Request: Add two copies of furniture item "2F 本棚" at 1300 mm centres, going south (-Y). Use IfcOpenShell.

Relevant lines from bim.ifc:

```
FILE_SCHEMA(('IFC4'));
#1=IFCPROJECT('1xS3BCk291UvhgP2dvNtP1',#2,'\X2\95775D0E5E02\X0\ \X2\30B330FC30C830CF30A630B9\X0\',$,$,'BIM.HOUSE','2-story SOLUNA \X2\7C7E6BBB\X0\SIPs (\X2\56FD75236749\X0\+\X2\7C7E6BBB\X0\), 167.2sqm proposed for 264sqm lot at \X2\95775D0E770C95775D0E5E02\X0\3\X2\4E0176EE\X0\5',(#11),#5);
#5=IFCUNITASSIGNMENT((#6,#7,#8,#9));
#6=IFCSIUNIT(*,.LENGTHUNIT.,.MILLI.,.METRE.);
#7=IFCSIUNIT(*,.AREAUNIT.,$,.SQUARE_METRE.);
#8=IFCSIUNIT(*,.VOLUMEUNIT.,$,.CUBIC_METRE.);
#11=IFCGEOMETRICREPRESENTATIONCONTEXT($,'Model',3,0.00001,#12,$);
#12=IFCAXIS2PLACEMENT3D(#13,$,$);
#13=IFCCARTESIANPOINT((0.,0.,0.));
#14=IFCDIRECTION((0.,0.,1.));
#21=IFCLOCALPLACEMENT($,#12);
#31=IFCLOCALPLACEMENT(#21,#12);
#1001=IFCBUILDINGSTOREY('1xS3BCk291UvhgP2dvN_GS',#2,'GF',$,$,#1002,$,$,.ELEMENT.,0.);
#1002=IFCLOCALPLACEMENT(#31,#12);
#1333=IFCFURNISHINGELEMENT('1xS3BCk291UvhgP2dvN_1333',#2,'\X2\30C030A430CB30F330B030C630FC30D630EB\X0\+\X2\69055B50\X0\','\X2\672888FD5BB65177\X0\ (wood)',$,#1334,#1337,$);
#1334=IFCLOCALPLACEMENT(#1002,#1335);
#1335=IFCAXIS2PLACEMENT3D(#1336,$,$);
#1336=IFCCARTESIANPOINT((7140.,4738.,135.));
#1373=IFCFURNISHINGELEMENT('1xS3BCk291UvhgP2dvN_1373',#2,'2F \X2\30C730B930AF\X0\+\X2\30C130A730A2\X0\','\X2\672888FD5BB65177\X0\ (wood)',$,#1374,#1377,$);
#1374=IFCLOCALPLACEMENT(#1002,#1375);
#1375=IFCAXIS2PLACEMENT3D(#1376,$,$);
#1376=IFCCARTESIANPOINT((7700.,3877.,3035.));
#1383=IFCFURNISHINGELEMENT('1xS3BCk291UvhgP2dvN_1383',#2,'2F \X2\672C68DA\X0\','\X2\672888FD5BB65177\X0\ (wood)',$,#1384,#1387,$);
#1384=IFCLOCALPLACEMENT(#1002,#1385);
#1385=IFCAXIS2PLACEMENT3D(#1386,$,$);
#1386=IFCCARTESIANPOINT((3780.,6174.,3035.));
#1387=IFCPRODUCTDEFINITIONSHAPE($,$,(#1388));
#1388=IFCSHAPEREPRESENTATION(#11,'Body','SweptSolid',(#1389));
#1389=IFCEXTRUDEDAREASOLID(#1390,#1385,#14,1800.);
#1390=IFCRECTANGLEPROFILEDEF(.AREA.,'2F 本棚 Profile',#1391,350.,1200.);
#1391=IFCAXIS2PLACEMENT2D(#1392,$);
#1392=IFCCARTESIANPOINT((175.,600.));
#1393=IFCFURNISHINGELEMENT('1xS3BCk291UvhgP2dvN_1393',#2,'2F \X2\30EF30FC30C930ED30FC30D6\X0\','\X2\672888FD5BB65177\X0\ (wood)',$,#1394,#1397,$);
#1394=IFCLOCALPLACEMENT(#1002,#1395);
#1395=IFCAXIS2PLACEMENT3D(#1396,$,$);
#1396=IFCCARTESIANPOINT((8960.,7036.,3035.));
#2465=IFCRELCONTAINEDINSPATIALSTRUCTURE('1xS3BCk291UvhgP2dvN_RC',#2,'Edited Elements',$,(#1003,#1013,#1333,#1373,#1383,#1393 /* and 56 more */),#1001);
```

```python
import numpy as np
import ifcopenshell
import ifcopenshell.api.geometry
import ifcopenshell.api.root
import ifcopenshell.util.element
import ifcopenshell.util.placement
import ifcopenshell.util.unit

model = ifcopenshell.open("bim.ifc")
unit_scale = ifcopenshell.util.unit.calculate_unit_scale(model)


def reuse_history(source, copy):
    """copy_class also copies each property set's owner history, people and application; keep the originals."""
    for rel in copy.IsDefinedBy:
        if rel.is_a("IfcRelDefinesByProperties") and (history := rel.RelatingPropertyDefinition.OwnerHistory):
            rel.RelatingPropertyDefinition.OwnerHistory = source.OwnerHistory
            ifcopenshell.util.element.remove_deep2(model, history)


source = model.by_guid("1xS3BCk291UvhgP2dvN_1383")
base = ifcopenshell.util.placement.get_local_placement(source.ObjectPlacement)
step = np.array([0.0, -1.0, 0.0]) * 1.3 / unit_scale

for i in range(1, 3):
    copy = ifcopenshell.api.root.copy_class(model, product=source)
    copy.Representation = ifcopenshell.util.element.copy_deep(
        model, source.Representation, exclude=["IfcGeometricRepresentationContext", "IfcRepresentationMap"]
    )
    reuse_history(source, copy)
    matrix = base.copy()
    matrix[:3, 3] += i * step
    print("added at", matrix[:3, 3].round(3) + 0.0)
    ifcopenshell.api.geometry.edit_object_placement(model, product=copy, matrix=matrix, is_si=False)

model.write("bim_rev.ifc")
```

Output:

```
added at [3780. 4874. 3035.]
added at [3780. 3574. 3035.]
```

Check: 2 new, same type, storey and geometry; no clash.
